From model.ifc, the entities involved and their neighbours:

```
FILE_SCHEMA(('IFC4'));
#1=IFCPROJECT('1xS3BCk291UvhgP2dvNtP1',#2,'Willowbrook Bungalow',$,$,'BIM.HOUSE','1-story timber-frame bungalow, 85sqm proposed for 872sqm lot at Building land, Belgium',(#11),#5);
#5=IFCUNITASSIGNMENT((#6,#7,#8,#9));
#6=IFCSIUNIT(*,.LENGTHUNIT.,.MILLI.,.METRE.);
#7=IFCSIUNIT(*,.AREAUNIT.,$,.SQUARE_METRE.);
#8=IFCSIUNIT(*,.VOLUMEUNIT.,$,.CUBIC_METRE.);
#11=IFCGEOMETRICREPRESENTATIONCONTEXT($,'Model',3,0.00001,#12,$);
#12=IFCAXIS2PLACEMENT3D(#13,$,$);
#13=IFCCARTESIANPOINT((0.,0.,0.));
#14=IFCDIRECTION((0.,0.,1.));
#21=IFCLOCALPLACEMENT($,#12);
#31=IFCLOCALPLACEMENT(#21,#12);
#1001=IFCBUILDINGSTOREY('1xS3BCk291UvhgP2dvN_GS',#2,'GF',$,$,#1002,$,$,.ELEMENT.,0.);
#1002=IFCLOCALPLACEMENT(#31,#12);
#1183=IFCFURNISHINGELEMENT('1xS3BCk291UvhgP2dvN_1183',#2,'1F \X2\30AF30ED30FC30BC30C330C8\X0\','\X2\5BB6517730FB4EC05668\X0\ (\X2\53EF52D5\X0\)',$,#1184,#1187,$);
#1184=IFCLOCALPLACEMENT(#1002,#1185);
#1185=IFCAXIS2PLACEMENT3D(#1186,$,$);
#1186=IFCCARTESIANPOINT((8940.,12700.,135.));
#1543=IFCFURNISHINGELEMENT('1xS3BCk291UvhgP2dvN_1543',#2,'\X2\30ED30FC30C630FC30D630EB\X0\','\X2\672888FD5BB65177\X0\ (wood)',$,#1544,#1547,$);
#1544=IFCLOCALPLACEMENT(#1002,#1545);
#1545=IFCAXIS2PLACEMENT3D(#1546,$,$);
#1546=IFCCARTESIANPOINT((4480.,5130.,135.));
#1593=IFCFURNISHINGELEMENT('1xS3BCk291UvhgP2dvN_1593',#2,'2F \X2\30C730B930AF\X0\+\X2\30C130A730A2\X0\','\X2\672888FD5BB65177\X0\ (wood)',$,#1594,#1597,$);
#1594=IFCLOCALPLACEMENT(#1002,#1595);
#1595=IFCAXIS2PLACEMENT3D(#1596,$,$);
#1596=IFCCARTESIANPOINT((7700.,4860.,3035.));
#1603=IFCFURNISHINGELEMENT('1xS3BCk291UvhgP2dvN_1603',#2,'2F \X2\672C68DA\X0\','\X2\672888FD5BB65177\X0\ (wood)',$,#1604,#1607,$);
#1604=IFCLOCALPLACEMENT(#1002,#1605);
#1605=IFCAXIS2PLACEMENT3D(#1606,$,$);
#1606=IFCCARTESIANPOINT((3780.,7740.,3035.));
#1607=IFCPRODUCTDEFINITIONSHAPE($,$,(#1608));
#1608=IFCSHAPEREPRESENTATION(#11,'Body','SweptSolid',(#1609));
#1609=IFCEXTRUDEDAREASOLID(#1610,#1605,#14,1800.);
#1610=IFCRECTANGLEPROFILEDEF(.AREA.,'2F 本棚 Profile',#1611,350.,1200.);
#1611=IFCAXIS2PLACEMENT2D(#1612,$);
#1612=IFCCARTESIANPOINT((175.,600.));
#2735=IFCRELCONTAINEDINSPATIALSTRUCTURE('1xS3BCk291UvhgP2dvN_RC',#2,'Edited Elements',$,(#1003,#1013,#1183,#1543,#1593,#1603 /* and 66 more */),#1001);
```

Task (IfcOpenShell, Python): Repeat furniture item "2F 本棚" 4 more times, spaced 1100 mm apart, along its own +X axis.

```python
import ifcopenshell
import ifcopenshell.api.geometry
import ifcopenshell.api.root
import ifcopenshell.util.element
import ifcopenshell.util.placement

model = ifcopenshell.open("model.ifc")


def reuse_history(source, copy):
    """copy_class also copies each property set's owner history, people and application; keep the originals."""
    for rel in copy.IsDefinedBy:
        if rel.is_a("IfcRelDefinesByProperties") and (history := rel.RelatingPropertyDefinition.OwnerHistory):
            rel.RelatingPropertyDefinition.OwnerHistory = source.OwnerHistory
            ifcopenshell.util.element.remove_deep2(model, history)


source = model.by_guid("1xS3BCk291UvhgP2dvN_1603")
base = ifcopenshell.util.placement.get_local_placement(source.ObjectPlacement)
step = base[:3, 0] * 1100.0

for i in range(1, 5):
    copy = ifcopenshell.api.root.copy_class(model, product=source)
    copy.Representation = ifcopenshell.util.element.copy_deep(
        model, source.Representation, exclude=["IfcGeometricRepresentationContext", "IfcRepresentationMap"]
    )
    reuse_history(source, copy)
    matrix = base.copy()
    matrix[:3, 3] += i * step
    print("added at", matrix[:3, 3].round(3) + 0.0)
    ifcopenshell.api.geometry.edit_object_placement(model, product=copy, matrix=matrix, is_si=False)

model.write("model_rev.ifc")
```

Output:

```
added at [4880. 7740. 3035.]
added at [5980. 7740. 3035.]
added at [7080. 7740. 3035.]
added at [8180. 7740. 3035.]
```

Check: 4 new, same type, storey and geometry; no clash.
